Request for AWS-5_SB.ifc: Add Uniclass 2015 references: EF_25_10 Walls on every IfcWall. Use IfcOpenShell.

First a look at what the model holds.

```python
import ifcopenshell

model = ifcopenshell.open("AWS-5_SB.ifc")
print(model.schema)
print("classifications:", [c.Name for c in model.by_type("IfcClassification")])
for ifc_class in ("IfcDoor", "IfcRoof", "IfcStair", "IfcWall", "IfcWindow"):
    print(ifc_class, len(model.by_type(ifc_class)))
```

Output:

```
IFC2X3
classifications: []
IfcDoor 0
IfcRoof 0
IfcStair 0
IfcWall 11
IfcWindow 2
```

```python
import ifcopenshell
import ifcopenshell.api.classification

model = ifcopenshell.open("AWS-5_SB.ifc")

# IFC2X3 requires Source and Edition and has no link from the project to the system.
system = model.create_entity("IfcClassification", Source="NBS", Edition="2015", Name="Uniclass 2015")

codes = {
    "IfcWall": ("EF_25_10", "Walls"),
}
for ifc_class, (code, name) in codes.items():
    products = model.by_type(ifc_class)
    ifcopenshell.api.classification.add_reference(
        model, products=products, classification=system, identification=code, name=name
    )
    print(code, len(products))

model.write("AWS-5_SB_updated.ifc")
```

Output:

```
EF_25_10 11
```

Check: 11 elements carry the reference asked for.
